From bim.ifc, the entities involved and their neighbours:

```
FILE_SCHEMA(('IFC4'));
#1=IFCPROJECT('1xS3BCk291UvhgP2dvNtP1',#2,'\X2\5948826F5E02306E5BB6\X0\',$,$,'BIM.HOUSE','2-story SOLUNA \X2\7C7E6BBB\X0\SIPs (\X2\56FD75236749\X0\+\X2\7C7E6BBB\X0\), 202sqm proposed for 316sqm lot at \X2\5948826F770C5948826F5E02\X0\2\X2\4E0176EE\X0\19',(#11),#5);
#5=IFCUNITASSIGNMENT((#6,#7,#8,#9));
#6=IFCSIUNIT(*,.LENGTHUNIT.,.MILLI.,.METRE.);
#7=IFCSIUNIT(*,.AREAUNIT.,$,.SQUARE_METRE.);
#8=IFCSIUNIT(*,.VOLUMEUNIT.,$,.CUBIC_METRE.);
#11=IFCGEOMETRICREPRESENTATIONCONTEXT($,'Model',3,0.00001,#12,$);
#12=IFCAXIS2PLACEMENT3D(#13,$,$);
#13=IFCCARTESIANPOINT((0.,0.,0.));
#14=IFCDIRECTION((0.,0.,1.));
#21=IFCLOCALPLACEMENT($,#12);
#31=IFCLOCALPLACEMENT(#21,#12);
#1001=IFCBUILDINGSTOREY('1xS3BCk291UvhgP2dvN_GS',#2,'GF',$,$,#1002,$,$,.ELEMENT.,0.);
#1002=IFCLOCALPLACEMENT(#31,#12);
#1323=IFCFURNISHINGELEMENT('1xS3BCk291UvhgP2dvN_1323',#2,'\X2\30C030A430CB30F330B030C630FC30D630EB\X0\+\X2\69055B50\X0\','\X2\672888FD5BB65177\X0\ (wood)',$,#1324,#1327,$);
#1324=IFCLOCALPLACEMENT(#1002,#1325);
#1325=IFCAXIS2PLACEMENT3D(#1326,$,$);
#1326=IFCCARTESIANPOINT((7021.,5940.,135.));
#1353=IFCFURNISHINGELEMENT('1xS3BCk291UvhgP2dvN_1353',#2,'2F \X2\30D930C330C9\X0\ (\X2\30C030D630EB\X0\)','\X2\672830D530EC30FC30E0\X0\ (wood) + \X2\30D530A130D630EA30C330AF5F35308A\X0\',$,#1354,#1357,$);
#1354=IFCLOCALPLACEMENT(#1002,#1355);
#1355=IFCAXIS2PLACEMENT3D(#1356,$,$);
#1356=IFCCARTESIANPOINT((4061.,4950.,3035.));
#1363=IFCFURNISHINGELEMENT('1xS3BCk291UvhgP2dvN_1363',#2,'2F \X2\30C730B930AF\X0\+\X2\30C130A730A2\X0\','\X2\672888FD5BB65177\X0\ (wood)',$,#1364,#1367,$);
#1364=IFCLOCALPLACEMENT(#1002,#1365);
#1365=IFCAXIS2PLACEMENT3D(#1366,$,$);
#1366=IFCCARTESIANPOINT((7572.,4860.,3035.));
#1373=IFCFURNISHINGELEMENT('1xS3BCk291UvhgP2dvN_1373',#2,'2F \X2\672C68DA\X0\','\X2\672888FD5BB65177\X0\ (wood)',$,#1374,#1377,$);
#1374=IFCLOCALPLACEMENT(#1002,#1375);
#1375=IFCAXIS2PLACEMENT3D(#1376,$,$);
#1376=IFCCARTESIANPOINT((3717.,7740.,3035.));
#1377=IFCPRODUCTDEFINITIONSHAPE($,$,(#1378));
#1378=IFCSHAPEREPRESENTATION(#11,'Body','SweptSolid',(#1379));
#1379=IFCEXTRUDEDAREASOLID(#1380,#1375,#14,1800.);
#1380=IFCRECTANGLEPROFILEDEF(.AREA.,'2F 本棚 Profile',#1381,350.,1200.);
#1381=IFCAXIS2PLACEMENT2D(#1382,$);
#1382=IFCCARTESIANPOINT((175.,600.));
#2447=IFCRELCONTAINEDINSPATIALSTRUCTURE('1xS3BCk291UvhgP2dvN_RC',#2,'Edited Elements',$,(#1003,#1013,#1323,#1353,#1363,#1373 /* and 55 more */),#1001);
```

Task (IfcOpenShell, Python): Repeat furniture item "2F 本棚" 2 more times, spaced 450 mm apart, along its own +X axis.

```python
import ifcopenshell
import ifcopenshell.api.geometry
import ifcopenshell.api.root
import ifcopenshell.util.element
import ifcopenshell.util.placement

model = ifcopenshell.open("bim.ifc")


def reuse_history(source, copy):
    """copy_class also copies each property set's owner history, people and application; keep the originals."""
    for rel in copy.IsDefinedBy:
        if rel.is_a("IfcRelDefinesByProperties") and (history := rel.RelatingPropertyDefinition.OwnerHistory):
            rel.RelatingPropertyDefinition.OwnerHistory = source.OwnerHistory
            ifcopenshell.util.element.remove_deep2(model, history)


source = model.by_guid("1xS3BCk291UvhgP2dvN_1373")
base = ifcopenshell.util.placement.get_local_placement(source.ObjectPlacement)
step = base[:3, 0] * 450.0

for i in range(1, 3):
    copy = ifcopenshell.api.root.copy_class(model, product=source)
    copy.Representation = ifcopenshell.util.element.copy_deep(
        model, source.Representation, exclude=["IfcGeometricRepresentationContext", "IfcRepresentationMap"]
    )
    reuse_history(source, copy)
    matrix = base.copy()
    matrix[:3, 3] += i * step
    print("added at", matrix[:3, 3].round(3) + 0.0)
    ifcopenshell.api.geometry.edit_object_placement(model, product=copy, matrix=matrix, is_si=False)

model.write("bim_rev.ifc")
```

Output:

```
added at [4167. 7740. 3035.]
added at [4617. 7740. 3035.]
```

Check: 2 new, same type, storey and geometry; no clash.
